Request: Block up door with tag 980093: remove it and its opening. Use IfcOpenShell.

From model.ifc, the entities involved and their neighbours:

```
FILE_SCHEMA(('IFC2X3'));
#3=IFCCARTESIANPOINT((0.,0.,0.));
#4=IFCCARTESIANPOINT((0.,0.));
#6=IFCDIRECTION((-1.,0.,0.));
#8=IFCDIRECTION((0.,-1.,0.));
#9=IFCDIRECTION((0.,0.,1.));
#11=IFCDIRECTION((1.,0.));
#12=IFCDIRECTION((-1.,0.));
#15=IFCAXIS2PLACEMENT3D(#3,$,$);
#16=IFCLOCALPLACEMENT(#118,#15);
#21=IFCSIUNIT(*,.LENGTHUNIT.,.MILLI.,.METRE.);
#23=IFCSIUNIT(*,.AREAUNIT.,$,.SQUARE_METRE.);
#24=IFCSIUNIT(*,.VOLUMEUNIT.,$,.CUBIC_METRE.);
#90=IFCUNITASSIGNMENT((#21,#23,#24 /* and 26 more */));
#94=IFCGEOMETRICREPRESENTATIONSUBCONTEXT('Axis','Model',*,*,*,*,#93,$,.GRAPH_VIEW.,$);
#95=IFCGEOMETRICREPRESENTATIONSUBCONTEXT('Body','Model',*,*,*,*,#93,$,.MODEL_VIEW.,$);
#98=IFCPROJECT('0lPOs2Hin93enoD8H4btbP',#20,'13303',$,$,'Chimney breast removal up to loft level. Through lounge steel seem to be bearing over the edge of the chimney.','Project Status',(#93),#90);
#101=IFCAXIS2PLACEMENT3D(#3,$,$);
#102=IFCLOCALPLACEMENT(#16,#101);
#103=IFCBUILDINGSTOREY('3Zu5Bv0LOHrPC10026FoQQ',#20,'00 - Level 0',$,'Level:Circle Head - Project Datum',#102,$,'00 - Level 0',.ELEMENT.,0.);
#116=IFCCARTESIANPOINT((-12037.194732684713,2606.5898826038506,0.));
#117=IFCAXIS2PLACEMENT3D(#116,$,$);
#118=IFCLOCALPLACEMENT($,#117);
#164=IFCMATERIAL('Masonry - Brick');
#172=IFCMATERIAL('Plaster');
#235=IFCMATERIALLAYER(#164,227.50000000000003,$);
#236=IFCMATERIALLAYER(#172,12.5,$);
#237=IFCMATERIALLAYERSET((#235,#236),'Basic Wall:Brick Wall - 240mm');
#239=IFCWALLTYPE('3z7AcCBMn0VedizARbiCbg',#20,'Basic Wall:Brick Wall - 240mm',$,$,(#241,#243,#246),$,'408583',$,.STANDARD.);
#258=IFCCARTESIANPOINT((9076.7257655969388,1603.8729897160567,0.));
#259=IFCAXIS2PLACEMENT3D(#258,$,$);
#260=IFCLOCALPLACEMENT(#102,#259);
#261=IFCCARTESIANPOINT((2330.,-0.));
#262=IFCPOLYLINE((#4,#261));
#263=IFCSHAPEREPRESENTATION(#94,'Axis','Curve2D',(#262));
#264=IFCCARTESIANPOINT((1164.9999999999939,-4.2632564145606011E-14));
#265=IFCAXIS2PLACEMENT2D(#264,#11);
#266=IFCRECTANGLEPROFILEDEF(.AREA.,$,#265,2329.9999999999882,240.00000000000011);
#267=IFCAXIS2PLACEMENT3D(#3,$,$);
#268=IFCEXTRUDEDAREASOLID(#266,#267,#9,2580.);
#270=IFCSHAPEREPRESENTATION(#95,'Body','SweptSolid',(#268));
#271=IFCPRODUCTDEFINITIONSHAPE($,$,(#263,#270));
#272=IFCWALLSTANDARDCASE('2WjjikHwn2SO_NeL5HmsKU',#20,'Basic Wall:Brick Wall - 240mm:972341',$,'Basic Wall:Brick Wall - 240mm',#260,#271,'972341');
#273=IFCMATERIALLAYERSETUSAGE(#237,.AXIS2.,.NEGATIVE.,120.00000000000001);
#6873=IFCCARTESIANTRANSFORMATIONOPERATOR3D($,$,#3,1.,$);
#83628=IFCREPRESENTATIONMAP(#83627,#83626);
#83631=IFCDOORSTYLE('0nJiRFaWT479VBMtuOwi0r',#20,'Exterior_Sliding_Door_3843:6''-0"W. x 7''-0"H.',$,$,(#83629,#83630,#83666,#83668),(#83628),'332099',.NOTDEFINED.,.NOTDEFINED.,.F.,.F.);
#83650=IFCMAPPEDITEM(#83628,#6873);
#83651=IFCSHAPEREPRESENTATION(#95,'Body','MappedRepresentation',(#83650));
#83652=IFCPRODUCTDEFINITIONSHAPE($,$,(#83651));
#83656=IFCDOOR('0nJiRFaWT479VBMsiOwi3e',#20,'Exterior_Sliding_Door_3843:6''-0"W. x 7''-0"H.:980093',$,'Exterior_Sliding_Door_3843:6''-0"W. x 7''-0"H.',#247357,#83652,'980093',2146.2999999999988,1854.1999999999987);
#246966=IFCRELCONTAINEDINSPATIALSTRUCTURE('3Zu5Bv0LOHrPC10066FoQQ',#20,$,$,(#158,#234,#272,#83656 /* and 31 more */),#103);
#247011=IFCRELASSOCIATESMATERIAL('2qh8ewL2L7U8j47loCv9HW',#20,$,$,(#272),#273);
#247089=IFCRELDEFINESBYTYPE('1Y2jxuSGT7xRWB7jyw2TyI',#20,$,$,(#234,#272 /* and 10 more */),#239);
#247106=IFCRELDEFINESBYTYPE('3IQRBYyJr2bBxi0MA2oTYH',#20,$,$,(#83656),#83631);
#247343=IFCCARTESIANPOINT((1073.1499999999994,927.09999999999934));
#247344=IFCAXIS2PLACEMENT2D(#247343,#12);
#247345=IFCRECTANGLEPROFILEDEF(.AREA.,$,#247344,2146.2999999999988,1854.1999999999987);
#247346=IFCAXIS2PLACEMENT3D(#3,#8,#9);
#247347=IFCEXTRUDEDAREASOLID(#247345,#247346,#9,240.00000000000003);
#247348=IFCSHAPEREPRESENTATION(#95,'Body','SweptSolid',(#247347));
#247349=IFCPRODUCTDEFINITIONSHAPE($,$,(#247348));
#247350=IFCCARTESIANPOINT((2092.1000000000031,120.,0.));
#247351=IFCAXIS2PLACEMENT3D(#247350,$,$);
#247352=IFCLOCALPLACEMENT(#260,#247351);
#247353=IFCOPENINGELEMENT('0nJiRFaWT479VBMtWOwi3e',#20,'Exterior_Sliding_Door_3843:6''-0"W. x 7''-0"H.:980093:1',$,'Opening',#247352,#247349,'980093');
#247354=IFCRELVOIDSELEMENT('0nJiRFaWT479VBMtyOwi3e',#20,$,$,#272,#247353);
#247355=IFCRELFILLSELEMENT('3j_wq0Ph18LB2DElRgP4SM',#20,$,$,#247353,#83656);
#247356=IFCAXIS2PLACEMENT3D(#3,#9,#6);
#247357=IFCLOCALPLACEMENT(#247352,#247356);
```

```python
import ifcopenshell
import ifcopenshell.api.feature
import ifcopenshell.api.root
import ifcopenshell.geom
import ifcopenshell.util.shape

model = ifcopenshell.open("model.ifc")
settings = ifcopenshell.geom.settings()


def volume(element):
    """Net volume in cubic metres, openings subtracted."""
    shape = ifcopenshell.geom.create_shape(settings, element)
    return ifcopenshell.util.shape.get_volume(shape.geometry)


door = model.by_id(83656)
opening = door.FillsVoids[0].RelatingOpeningElement
wall = opening.VoidsElements[0].RelatingBuildingElement
before = volume(wall)

ifcopenshell.api.root.remove_product(model, product=door)
ifcopenshell.api.feature.remove_feature(model, feature=opening)

after = volume(wall)

print(f"wall volume {before:.3f} -> {after:.3f} m3")

model.write("model_edited.ifc")
```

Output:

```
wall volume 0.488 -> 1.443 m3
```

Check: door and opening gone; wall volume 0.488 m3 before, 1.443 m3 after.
